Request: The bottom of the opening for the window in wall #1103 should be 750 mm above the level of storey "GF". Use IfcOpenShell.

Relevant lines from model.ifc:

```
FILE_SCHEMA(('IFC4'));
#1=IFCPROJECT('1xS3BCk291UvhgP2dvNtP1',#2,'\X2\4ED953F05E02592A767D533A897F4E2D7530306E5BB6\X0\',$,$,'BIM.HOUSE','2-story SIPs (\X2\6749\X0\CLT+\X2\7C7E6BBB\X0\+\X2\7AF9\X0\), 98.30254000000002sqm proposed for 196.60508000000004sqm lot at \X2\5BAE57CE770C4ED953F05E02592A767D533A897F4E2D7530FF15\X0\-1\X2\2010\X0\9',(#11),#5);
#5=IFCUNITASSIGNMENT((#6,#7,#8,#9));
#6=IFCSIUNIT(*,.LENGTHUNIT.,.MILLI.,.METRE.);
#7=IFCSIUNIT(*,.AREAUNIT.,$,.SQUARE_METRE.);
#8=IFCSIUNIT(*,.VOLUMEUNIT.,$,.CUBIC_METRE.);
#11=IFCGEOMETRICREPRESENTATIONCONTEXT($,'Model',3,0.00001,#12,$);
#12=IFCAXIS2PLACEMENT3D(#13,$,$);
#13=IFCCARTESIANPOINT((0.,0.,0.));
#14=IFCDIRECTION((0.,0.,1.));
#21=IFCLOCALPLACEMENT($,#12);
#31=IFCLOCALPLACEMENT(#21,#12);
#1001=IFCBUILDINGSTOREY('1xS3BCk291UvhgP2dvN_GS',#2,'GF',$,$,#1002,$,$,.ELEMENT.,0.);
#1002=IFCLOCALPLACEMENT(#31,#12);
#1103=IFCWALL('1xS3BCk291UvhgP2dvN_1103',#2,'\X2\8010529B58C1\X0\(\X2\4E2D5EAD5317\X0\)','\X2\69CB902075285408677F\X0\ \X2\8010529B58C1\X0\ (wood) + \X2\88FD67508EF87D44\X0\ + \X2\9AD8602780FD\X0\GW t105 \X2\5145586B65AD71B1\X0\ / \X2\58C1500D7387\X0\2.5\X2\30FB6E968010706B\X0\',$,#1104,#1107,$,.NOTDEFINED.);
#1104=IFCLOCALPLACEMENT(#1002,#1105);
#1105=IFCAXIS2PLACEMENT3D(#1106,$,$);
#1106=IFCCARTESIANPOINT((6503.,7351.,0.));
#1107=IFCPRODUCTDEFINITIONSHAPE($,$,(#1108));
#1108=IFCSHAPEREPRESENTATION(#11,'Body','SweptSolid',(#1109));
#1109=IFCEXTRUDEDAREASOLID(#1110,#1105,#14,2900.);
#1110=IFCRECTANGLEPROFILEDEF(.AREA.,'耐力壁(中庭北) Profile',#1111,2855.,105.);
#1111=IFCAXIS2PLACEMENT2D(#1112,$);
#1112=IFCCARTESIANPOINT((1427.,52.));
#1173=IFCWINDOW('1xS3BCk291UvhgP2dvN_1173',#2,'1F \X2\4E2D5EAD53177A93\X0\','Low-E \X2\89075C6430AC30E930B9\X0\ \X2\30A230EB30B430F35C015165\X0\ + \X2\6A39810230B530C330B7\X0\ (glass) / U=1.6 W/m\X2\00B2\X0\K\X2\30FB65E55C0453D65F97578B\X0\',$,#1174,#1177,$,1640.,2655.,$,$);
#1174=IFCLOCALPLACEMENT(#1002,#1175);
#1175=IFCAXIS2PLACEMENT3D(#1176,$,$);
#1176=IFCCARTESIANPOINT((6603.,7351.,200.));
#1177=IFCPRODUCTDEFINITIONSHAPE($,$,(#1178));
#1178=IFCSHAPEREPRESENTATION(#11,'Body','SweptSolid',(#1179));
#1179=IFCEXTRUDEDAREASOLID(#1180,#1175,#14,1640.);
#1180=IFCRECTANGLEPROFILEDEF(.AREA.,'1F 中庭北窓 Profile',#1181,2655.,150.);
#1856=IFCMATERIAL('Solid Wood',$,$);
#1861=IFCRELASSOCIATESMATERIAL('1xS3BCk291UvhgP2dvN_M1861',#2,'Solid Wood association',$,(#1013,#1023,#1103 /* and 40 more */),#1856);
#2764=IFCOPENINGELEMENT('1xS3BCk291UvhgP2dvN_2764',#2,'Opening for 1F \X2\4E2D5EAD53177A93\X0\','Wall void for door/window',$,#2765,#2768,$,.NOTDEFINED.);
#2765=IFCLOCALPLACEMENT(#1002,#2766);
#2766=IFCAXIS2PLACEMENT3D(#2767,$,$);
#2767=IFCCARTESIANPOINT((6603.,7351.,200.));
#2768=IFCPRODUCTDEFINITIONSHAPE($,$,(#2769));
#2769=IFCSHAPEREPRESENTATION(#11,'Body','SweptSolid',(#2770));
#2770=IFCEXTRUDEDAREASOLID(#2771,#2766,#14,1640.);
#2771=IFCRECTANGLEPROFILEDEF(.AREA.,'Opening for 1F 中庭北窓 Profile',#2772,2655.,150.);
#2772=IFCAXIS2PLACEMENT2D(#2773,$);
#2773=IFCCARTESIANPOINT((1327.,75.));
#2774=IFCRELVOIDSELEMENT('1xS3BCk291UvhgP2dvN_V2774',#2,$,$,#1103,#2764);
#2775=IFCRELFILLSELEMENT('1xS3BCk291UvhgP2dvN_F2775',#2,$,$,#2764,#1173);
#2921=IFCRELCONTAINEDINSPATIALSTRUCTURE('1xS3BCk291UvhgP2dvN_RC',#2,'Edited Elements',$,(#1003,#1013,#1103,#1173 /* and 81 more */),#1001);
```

```python
import numpy as np
import ifcopenshell
import ifcopenshell.api.geometry
import ifcopenshell.geom
import ifcopenshell.util.element
import ifcopenshell.util.placement
import ifcopenshell.util.shape
import ifcopenshell.util.unit

model = ifcopenshell.open("model.ifc")
unit_scale = ifcopenshell.util.unit.calculate_unit_scale(model)

window = model.by_guid("1xS3BCk291UvhgP2dvN_1173")
opening = window.FillsVoids[0].RelatingOpeningElement
storey = ifcopenshell.util.element.get_container(window, ifc_class="IfcBuildingStorey")
level = ifcopenshell.util.placement.get_local_placement(storey.ObjectPlacement)[2, 3]

# The opening's origin need not be at the sill, so measure its lowest point.
shape = ifcopenshell.geom.create_shape(ifcopenshell.geom.settings(), opening)
bottom = ifcopenshell.util.shape.get_shape_bottom_elevation(shape, shape.geometry) / unit_scale
dz = level + 0.75 / unit_scale - bottom

shift = np.array([0.0, 0.0, dz])
# The window is not placed relative to its opening, so move both.
for product in (opening, window):
    matrix = ifcopenshell.util.placement.get_local_placement(product.ObjectPlacement)
    matrix[:3, 3] += shift
    ifcopenshell.api.geometry.edit_object_placement(model, product=product, matrix=matrix, is_si=False)

print(f"moved by {dz * unit_scale:+.3f} m")

model.write("model_rev.ifc")
```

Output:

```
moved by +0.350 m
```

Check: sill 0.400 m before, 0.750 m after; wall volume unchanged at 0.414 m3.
